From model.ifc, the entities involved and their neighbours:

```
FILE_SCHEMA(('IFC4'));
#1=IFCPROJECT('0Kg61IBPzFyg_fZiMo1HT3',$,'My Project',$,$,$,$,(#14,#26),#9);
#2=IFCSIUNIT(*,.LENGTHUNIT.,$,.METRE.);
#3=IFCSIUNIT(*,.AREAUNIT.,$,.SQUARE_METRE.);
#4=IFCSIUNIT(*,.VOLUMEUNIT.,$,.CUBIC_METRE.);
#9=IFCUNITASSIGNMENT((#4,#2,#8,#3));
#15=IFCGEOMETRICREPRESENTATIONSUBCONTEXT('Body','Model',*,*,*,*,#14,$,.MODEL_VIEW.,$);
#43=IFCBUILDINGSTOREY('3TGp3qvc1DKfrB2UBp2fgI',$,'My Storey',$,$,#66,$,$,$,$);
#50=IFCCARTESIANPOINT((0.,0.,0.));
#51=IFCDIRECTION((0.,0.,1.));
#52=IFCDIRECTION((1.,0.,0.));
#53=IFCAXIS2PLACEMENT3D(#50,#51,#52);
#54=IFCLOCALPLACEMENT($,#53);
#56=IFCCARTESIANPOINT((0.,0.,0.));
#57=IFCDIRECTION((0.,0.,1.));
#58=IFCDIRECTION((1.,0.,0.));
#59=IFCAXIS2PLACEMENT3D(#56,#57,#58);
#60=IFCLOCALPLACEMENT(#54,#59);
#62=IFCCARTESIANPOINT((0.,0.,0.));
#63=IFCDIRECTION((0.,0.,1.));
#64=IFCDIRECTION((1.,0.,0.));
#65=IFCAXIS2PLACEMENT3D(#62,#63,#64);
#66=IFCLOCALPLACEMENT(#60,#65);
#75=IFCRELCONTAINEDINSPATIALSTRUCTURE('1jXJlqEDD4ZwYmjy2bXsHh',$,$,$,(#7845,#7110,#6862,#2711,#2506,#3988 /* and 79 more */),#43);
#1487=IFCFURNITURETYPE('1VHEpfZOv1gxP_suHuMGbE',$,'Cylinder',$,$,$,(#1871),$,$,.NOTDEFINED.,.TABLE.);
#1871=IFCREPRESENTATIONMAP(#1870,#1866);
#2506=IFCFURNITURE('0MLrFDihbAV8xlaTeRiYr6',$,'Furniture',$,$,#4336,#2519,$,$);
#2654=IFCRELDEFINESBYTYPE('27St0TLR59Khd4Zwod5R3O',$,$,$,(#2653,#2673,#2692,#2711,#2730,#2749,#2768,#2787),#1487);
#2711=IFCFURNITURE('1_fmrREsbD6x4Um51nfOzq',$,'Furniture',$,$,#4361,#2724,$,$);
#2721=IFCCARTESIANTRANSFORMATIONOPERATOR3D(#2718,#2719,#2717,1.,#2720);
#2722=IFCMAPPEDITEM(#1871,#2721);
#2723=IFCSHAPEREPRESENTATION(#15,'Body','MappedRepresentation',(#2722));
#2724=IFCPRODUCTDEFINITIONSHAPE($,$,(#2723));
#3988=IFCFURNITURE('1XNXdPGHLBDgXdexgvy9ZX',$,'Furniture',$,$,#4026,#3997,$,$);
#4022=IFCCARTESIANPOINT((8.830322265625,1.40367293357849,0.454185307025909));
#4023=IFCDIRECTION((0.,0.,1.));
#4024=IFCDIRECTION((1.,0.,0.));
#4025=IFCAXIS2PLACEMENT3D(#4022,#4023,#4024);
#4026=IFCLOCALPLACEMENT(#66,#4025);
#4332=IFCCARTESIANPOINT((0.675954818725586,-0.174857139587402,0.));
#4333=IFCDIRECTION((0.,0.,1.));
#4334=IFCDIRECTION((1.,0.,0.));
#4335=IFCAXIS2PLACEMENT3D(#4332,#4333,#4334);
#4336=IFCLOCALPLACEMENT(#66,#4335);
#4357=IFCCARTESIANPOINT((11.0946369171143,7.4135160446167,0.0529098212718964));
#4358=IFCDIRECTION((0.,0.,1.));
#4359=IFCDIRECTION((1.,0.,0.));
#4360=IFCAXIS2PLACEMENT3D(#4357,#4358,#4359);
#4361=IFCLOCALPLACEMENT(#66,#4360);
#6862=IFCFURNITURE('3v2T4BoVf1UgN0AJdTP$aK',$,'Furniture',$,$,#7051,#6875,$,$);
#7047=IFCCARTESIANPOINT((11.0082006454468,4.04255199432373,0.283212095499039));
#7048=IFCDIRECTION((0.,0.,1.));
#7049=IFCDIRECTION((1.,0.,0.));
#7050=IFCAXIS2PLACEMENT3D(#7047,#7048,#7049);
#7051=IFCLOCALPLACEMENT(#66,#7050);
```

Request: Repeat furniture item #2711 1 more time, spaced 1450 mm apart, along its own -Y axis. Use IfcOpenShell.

```python
import ifcopenshell
import ifcopenshell.api.geometry
import ifcopenshell.api.root
import ifcopenshell.util.element
import ifcopenshell.util.placement

model = ifcopenshell.open("model.ifc")

source = model.by_guid("1_fmrREsbD6x4Um51nfOzq")
base = ifcopenshell.util.placement.get_local_placement(source.ObjectPlacement)
step = -base[:3, 1] * 1.45

for i in range(1, 2):
    copy = ifcopenshell.api.root.copy_class(model, product=source)
    copy.Representation = ifcopenshell.util.element.copy_deep(
        model, source.Representation, exclude=["IfcGeometricRepresentationContext", "IfcRepresentationMap"]
    )
    matrix = base.copy()
    matrix[:3, 3] += i * step
    print("added at", matrix[:3, 3].round(3) + 0.0)
    ifcopenshell.api.geometry.edit_object_placement(model, product=copy, matrix=matrix, is_si=False)

model.write("model_rev.ifc")
```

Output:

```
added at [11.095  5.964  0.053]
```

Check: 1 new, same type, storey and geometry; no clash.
